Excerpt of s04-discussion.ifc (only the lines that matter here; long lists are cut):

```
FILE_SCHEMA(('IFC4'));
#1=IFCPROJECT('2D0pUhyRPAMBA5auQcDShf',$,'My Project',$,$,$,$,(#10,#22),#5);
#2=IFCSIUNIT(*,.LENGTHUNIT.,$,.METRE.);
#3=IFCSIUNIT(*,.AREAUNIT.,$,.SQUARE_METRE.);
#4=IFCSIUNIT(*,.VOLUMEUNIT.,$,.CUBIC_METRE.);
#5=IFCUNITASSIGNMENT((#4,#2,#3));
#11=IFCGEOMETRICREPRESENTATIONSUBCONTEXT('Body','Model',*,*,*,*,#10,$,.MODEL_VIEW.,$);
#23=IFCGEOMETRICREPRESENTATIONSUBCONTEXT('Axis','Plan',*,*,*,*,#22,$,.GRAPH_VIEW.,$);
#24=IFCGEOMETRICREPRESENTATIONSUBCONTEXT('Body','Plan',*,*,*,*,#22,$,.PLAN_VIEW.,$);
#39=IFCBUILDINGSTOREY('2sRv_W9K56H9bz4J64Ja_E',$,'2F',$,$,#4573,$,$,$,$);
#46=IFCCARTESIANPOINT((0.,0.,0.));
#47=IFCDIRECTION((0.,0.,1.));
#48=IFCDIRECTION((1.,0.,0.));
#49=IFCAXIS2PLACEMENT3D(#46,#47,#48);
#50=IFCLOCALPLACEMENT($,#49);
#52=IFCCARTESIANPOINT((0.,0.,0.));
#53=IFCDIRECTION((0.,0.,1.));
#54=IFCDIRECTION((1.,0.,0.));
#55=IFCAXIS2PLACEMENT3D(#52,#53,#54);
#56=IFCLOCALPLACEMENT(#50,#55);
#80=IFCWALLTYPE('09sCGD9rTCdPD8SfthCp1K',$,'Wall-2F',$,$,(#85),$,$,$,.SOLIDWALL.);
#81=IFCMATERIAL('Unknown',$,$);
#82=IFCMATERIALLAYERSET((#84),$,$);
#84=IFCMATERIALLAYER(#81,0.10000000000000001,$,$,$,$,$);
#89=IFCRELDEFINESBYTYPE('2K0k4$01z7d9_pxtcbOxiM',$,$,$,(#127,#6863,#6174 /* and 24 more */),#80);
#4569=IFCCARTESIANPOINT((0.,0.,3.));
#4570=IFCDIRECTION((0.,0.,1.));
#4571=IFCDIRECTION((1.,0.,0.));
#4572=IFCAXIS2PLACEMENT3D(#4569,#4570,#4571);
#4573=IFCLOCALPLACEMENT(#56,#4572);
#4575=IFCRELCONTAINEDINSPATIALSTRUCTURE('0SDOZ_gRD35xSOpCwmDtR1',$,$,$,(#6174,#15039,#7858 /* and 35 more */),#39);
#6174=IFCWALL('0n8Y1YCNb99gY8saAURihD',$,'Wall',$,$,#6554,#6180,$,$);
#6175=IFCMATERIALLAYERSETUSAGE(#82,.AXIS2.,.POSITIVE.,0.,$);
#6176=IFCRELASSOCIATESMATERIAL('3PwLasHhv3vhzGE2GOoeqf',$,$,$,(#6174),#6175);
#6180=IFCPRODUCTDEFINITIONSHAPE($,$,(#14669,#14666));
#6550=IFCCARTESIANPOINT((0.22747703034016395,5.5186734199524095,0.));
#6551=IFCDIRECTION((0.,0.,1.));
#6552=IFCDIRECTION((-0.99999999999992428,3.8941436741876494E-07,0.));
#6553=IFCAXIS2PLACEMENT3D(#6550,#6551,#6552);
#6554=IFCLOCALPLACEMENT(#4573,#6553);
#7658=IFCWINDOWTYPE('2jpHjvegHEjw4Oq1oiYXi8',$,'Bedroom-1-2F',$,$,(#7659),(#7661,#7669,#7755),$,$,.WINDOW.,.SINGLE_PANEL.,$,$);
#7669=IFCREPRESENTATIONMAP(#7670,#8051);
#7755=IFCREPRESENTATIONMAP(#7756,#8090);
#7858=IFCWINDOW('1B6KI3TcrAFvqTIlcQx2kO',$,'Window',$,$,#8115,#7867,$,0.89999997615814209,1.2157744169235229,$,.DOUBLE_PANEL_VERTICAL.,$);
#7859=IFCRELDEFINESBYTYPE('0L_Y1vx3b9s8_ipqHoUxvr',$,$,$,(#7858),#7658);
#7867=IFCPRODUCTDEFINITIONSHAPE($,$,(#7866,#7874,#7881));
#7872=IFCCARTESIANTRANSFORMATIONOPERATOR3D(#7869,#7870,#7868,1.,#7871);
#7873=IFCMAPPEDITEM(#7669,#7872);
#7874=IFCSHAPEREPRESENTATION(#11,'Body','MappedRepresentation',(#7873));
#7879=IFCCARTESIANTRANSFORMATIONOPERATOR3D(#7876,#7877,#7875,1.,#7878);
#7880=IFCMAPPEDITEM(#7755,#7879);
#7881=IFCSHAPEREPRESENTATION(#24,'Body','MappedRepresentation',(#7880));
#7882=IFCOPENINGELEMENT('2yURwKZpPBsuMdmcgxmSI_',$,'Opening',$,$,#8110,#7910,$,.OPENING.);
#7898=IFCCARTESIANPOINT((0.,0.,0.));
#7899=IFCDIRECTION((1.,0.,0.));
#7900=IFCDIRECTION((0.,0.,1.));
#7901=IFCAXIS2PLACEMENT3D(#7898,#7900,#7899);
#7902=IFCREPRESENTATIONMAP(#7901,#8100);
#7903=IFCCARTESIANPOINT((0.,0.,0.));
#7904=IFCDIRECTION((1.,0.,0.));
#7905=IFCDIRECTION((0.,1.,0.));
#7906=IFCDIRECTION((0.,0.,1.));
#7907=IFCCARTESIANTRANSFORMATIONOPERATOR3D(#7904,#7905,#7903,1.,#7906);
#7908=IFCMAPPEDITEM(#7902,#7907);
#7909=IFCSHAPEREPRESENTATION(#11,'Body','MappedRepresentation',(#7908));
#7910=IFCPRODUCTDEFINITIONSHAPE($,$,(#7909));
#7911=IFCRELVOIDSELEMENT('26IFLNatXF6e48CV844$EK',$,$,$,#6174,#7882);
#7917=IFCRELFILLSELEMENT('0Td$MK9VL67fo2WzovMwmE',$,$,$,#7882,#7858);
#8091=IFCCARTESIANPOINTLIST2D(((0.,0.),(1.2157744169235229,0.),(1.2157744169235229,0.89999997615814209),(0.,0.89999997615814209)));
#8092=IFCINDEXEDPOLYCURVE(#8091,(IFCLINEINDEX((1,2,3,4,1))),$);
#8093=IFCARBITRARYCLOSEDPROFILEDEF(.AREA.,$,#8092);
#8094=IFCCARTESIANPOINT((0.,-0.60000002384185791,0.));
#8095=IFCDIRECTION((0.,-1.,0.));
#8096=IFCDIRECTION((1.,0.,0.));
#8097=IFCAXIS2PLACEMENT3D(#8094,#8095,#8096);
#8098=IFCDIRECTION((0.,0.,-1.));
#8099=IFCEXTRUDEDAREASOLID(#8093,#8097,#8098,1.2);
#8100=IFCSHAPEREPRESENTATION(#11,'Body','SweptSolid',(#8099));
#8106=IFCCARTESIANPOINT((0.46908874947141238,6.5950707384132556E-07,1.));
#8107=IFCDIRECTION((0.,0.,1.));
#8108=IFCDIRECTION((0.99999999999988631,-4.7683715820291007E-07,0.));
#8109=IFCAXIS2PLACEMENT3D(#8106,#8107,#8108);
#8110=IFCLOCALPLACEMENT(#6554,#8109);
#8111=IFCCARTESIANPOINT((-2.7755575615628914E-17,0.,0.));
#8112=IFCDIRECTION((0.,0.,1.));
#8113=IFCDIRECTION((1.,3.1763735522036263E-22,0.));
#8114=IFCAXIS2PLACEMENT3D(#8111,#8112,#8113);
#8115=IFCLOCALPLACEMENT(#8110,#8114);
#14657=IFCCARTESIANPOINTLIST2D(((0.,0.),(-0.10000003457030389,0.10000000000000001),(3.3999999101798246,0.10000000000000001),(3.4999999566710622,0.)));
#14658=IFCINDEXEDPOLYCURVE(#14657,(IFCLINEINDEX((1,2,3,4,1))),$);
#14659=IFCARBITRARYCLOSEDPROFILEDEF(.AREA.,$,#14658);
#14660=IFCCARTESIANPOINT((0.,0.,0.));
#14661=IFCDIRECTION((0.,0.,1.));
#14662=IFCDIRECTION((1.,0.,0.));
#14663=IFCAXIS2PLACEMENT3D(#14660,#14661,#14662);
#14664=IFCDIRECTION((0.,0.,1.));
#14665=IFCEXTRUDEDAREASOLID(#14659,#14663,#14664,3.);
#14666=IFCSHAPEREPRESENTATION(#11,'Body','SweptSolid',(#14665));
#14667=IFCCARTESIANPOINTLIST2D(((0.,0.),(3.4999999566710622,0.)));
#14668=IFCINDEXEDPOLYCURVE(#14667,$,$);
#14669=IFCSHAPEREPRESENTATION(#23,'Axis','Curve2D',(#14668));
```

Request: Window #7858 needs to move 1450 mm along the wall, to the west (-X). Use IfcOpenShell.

```python
import ifcopenshell
import ifcopenshell.api.geometry
import ifcopenshell.util.placement
import ifcopenshell.util.unit

model = ifcopenshell.open("s04-discussion.ifc")
unit_scale = ifcopenshell.util.unit.calculate_unit_scale(model)

window = model.by_id(7858)
opening = window.FillsVoids[0].RelatingOpeningElement
wall = opening.VoidsElements[0].RelatingBuildingElement

wall_matrix = ifcopenshell.util.placement.get_local_placement(wall.ObjectPlacement)
shift = wall_matrix[:3, 0] * 1.45 / unit_scale
before = ifcopenshell.util.placement.get_local_placement(window.ObjectPlacement)[:3, 3].copy()

# The window is placed relative to its opening, so it follows when the opening moves.
matrix = ifcopenshell.util.placement.get_local_placement(opening.ObjectPlacement)
matrix[:3, 3] += shift
ifcopenshell.api.geometry.edit_object_placement(
    model, product=opening, matrix=matrix, is_si=False, should_transform_children=True
)

after = ifcopenshell.util.placement.get_local_placement(window.ObjectPlacement)[:3, 3]
print("window moved by", (after - before).round(3) + 0.0)

model.write("s04-discussion_rev.ifc")
```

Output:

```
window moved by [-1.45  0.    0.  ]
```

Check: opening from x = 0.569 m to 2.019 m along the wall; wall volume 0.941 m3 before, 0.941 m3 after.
